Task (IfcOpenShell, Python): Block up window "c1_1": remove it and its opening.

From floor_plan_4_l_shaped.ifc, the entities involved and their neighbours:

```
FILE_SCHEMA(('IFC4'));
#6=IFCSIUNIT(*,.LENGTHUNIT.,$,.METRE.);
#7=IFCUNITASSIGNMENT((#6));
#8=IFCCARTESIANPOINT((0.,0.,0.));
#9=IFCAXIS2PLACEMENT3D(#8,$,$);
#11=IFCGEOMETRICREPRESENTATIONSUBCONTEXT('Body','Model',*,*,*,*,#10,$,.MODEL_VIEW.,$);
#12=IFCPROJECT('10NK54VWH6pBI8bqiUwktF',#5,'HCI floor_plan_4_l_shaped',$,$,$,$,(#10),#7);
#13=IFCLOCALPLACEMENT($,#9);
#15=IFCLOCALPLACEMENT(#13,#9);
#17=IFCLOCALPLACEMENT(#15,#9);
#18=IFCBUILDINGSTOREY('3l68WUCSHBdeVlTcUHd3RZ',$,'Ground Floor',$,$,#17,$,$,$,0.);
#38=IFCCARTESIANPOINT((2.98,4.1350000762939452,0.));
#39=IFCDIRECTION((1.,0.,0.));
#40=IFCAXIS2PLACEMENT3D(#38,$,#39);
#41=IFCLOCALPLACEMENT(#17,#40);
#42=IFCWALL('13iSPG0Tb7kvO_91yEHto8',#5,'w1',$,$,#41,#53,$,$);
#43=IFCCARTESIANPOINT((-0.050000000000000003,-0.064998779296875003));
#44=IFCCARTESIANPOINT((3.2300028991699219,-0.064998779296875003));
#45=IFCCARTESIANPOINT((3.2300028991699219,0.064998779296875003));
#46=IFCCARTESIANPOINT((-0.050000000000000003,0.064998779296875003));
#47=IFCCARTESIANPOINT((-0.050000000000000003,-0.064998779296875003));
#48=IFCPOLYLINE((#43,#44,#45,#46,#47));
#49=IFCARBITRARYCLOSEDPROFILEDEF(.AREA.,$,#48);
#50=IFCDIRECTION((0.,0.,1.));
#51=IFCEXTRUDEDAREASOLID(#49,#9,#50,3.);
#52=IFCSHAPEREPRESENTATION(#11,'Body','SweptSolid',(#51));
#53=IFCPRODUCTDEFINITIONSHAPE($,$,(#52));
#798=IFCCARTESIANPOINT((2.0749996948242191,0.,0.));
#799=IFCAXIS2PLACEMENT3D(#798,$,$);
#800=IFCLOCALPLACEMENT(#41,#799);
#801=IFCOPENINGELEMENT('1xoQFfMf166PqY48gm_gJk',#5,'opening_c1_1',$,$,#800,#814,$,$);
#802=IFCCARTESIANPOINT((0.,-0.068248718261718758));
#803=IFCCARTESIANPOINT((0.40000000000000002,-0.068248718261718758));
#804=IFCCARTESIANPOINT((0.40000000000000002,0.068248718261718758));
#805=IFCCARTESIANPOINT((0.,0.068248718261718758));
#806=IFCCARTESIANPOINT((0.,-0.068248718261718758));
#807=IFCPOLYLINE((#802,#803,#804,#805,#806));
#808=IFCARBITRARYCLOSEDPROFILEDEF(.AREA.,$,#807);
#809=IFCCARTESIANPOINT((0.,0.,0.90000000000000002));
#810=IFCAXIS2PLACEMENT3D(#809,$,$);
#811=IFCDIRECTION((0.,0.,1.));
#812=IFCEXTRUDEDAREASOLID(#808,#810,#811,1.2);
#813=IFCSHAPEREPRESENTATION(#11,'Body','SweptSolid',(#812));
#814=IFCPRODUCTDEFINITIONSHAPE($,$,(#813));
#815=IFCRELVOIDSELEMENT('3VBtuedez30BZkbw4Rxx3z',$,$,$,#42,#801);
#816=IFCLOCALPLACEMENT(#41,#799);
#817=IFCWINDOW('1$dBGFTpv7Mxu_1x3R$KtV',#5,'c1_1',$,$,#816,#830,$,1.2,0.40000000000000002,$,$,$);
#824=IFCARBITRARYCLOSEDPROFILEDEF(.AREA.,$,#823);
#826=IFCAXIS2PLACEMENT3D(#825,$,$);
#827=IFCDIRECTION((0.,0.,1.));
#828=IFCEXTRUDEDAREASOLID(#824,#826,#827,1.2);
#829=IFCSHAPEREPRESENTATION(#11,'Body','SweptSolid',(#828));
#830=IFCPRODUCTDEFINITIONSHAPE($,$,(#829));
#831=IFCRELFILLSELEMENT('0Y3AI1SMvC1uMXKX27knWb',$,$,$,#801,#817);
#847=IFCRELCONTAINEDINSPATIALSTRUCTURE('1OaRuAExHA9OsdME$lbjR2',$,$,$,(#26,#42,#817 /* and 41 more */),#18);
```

```python
import ifcopenshell
import ifcopenshell.api.feature
import ifcopenshell.api.root
import ifcopenshell.geom
import ifcopenshell.util.shape

model = ifcopenshell.open("floor_plan_4_l_shaped.ifc")
settings = ifcopenshell.geom.settings()


def volume(element):
    """Net volume in cubic metres, openings subtracted."""
    shape = ifcopenshell.geom.create_shape(settings, element)
    return ifcopenshell.util.shape.get_volume(shape.geometry)


window = model.by_guid("1$dBGFTpv7Mxu_1x3R$KtV")
opening = window.FillsVoids[0].RelatingOpeningElement
wall = opening.VoidsElements[0].RelatingBuildingElement
before = volume(wall)

ifcopenshell.api.root.remove_product(model, product=window)
ifcopenshell.api.feature.remove_feature(model, feature=opening)

after = volume(wall)

print(f"wall volume {before:.3f} -> {after:.3f} m3")

model.write("floor_plan_4_l_shaped_v2.ifc")
```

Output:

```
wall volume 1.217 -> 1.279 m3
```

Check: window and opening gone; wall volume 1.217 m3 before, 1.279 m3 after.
